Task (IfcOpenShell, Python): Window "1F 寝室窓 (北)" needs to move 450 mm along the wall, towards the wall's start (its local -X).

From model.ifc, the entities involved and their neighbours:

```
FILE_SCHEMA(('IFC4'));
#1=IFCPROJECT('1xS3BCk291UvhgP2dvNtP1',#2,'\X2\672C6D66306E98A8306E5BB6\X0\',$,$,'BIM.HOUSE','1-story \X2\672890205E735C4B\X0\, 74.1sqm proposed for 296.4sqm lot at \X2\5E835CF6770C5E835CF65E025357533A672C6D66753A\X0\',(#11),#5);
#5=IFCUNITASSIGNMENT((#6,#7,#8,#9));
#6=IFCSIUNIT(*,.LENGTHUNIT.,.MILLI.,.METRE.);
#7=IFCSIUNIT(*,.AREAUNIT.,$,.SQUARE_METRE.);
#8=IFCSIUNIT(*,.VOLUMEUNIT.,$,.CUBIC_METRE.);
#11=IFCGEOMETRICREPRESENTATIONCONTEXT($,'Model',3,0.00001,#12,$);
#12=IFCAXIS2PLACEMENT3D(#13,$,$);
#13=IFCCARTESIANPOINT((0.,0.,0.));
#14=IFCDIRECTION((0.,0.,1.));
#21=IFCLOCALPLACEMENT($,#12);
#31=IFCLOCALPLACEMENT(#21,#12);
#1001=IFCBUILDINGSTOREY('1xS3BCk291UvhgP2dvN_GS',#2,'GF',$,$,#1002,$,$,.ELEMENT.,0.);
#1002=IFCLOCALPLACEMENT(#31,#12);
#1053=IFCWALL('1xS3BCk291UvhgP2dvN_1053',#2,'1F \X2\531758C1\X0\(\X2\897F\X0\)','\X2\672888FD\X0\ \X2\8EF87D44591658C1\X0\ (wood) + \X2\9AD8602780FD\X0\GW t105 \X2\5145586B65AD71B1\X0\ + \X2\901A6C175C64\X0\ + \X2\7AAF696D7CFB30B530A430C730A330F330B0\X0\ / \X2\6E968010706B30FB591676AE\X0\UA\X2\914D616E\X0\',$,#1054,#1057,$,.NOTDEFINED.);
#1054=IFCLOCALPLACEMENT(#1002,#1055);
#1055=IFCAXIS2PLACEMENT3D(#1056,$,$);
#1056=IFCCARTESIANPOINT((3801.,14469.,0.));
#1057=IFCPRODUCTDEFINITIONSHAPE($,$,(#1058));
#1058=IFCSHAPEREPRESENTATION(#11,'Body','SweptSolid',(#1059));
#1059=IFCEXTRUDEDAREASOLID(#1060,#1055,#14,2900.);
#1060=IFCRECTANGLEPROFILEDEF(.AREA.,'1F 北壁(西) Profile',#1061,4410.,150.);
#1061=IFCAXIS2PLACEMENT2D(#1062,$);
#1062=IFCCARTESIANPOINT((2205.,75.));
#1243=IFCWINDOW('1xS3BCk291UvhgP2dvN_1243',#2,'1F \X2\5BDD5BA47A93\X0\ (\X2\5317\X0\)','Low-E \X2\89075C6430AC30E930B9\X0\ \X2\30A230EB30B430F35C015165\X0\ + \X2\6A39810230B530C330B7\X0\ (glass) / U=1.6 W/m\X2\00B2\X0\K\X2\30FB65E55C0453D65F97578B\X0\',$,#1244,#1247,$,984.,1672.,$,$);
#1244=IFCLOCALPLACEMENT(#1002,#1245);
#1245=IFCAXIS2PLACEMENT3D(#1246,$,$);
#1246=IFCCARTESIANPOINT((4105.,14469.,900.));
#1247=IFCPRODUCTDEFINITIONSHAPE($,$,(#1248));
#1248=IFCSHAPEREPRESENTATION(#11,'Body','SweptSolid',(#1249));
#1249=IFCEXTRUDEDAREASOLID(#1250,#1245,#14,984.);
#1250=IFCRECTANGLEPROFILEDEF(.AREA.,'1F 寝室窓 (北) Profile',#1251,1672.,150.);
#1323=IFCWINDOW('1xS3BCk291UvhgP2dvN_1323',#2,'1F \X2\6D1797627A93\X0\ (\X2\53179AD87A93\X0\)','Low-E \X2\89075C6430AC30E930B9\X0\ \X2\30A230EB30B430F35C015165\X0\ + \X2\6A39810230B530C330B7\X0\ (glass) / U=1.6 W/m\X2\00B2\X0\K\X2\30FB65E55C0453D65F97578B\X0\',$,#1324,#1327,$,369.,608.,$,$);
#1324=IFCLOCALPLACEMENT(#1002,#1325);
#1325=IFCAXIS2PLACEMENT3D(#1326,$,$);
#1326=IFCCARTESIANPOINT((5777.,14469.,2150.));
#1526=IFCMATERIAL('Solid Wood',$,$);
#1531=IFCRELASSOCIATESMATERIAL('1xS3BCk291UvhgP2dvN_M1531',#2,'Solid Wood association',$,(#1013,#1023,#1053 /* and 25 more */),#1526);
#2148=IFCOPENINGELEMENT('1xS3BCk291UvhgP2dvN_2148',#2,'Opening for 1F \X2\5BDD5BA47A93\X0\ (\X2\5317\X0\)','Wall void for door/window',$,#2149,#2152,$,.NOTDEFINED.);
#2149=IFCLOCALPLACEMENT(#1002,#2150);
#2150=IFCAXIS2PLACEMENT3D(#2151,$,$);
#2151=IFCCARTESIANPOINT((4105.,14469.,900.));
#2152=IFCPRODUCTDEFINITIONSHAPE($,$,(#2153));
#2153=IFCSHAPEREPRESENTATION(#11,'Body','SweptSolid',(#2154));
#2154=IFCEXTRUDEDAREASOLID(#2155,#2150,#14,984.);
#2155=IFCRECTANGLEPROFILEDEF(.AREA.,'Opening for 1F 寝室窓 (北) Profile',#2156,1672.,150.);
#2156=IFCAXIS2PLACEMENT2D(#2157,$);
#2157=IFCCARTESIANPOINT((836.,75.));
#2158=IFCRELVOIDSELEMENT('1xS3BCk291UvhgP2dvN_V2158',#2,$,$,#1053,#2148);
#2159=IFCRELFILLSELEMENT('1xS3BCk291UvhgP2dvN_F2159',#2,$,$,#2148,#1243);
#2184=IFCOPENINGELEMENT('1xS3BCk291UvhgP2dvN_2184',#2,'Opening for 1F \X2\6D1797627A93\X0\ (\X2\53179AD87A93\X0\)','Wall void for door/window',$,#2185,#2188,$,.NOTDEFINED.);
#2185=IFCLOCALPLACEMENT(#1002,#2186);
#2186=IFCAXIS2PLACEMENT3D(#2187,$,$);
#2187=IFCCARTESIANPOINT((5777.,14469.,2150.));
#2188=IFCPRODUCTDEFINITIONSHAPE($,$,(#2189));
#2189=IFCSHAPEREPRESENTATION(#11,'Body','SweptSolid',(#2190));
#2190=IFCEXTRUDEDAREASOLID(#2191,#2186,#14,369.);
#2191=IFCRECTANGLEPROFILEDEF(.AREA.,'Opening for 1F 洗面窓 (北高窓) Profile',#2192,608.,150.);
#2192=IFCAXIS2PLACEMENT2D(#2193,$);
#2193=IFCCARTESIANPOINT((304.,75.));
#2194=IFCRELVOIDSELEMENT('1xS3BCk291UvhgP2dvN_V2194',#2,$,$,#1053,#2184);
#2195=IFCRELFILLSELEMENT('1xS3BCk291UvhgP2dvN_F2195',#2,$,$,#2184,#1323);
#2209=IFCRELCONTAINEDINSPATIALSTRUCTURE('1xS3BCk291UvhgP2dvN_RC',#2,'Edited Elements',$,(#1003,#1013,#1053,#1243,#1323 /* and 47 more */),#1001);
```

```python
import ifcopenshell
import ifcopenshell.api.geometry
import ifcopenshell.util.placement
import ifcopenshell.util.unit

model = ifcopenshell.open("model.ifc")
unit_scale = ifcopenshell.util.unit.calculate_unit_scale(model)

window = model.by_guid("1xS3BCk291UvhgP2dvN_1243")
opening = window.FillsVoids[0].RelatingOpeningElement
wall = opening.VoidsElements[0].RelatingBuildingElement

wall_matrix = ifcopenshell.util.placement.get_local_placement(wall.ObjectPlacement)
shift = wall_matrix[:3, 0] * -0.45 / unit_scale
before = ifcopenshell.util.placement.get_local_placement(window.ObjectPlacement)[:3, 3].copy()

# The window is not placed relative to its opening, so move both.
for product in (opening, window):
    matrix = ifcopenshell.util.placement.get_local_placement(product.ObjectPlacement)
    matrix[:3, 3] += shift
    ifcopenshell.api.geometry.edit_object_placement(model, product=product, matrix=matrix, is_si=False)

after = ifcopenshell.util.placement.get_local_placement(window.ObjectPlacement)[:3, 3]
print("window moved by", (after - before).round(3) + 0.0)

model.write("model_rev.ifc")
```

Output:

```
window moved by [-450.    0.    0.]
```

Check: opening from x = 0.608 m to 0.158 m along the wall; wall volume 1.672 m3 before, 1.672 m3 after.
